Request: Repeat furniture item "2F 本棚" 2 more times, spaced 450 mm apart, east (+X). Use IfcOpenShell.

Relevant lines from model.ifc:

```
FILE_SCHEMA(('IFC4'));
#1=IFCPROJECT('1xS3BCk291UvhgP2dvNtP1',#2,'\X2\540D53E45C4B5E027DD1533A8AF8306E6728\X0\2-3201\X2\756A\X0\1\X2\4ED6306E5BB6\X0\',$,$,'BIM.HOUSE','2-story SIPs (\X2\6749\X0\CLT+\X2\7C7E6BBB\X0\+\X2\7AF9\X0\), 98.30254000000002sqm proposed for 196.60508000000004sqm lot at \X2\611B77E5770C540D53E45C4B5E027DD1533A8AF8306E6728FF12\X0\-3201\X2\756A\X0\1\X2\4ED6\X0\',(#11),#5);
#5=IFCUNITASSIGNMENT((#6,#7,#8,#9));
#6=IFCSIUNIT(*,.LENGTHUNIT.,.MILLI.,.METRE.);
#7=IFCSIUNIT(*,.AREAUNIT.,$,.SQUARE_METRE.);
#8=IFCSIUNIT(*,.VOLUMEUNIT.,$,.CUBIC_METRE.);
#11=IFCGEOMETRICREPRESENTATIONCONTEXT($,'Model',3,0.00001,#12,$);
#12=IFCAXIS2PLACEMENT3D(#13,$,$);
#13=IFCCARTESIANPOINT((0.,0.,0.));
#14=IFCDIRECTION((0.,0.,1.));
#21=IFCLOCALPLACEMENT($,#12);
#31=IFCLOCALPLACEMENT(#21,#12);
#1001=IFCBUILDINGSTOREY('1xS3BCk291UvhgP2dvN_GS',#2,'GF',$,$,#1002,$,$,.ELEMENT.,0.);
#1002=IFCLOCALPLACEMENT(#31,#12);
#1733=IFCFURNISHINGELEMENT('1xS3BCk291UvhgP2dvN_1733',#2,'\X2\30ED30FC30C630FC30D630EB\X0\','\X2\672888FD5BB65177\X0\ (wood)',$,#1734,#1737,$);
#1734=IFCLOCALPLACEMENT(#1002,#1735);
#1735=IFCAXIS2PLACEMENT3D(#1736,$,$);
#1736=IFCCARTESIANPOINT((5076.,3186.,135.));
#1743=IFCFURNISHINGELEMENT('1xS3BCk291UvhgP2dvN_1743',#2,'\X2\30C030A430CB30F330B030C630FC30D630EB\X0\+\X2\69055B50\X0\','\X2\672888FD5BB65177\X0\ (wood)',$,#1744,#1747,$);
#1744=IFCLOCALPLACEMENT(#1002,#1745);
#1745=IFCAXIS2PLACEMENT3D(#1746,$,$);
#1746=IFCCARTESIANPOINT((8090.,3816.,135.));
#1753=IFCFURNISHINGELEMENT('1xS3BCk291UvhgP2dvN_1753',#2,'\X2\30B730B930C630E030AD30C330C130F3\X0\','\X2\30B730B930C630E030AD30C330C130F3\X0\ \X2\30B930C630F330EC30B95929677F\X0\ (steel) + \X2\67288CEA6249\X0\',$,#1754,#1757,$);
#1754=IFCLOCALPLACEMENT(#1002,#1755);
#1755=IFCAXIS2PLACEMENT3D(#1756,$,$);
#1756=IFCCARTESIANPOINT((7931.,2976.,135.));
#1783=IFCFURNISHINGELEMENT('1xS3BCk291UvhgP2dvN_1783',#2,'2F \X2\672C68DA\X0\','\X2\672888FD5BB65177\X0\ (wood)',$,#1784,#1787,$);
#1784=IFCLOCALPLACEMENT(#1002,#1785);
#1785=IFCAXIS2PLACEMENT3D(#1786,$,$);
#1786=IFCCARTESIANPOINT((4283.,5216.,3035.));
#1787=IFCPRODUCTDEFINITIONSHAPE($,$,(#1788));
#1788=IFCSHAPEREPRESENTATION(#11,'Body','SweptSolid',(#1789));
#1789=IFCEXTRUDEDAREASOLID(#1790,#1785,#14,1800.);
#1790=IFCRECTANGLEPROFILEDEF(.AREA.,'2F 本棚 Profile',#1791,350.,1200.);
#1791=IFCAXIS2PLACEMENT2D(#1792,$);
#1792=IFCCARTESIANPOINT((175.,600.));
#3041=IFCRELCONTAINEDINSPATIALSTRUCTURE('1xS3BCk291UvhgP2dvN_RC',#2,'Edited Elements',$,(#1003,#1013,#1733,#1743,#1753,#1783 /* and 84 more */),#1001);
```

```python
import numpy as np
import ifcopenshell
import ifcopenshell.api.geometry
import ifcopenshell.api.root
import ifcopenshell.util.element
import ifcopenshell.util.placement
import ifcopenshell.util.unit

model = ifcopenshell.open("model.ifc")
unit_scale = ifcopenshell.util.unit.calculate_unit_scale(model)


def reuse_history(source, copy):
    """copy_class also copies each property set's owner history, people and application; keep the originals."""
    for rel in copy.IsDefinedBy:
        if rel.is_a("IfcRelDefinesByProperties") and (history := rel.RelatingPropertyDefinition.OwnerHistory):
            rel.RelatingPropertyDefinition.OwnerHistory = source.OwnerHistory
            ifcopenshell.util.element.remove_deep2(model, history)


source = model.by_guid("1xS3BCk291UvhgP2dvN_1783")
base = ifcopenshell.util.placement.get_local_placement(source.ObjectPlacement)
step = np.array([1.0, 0.0, 0.0]) * 0.45 / unit_scale

for i in range(1, 3):
    copy = ifcopenshell.api.root.copy_class(model, product=source)
    copy.Representation = ifcopenshell.util.element.copy_deep(
        model, source.Representation, exclude=["IfcGeometricRepresentationContext", "IfcRepresentationMap"]
    )
    reuse_history(source, copy)
    matrix = base.copy()
    matrix[:3, 3] += i * step
    print("added at", matrix[:3, 3].round(3) + 0.0)
    ifcopenshell.api.geometry.edit_object_placement(model, product=copy, matrix=matrix, is_si=False)

model.write("model_updated.ifc")
```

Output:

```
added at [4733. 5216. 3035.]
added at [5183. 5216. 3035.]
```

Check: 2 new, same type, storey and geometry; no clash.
